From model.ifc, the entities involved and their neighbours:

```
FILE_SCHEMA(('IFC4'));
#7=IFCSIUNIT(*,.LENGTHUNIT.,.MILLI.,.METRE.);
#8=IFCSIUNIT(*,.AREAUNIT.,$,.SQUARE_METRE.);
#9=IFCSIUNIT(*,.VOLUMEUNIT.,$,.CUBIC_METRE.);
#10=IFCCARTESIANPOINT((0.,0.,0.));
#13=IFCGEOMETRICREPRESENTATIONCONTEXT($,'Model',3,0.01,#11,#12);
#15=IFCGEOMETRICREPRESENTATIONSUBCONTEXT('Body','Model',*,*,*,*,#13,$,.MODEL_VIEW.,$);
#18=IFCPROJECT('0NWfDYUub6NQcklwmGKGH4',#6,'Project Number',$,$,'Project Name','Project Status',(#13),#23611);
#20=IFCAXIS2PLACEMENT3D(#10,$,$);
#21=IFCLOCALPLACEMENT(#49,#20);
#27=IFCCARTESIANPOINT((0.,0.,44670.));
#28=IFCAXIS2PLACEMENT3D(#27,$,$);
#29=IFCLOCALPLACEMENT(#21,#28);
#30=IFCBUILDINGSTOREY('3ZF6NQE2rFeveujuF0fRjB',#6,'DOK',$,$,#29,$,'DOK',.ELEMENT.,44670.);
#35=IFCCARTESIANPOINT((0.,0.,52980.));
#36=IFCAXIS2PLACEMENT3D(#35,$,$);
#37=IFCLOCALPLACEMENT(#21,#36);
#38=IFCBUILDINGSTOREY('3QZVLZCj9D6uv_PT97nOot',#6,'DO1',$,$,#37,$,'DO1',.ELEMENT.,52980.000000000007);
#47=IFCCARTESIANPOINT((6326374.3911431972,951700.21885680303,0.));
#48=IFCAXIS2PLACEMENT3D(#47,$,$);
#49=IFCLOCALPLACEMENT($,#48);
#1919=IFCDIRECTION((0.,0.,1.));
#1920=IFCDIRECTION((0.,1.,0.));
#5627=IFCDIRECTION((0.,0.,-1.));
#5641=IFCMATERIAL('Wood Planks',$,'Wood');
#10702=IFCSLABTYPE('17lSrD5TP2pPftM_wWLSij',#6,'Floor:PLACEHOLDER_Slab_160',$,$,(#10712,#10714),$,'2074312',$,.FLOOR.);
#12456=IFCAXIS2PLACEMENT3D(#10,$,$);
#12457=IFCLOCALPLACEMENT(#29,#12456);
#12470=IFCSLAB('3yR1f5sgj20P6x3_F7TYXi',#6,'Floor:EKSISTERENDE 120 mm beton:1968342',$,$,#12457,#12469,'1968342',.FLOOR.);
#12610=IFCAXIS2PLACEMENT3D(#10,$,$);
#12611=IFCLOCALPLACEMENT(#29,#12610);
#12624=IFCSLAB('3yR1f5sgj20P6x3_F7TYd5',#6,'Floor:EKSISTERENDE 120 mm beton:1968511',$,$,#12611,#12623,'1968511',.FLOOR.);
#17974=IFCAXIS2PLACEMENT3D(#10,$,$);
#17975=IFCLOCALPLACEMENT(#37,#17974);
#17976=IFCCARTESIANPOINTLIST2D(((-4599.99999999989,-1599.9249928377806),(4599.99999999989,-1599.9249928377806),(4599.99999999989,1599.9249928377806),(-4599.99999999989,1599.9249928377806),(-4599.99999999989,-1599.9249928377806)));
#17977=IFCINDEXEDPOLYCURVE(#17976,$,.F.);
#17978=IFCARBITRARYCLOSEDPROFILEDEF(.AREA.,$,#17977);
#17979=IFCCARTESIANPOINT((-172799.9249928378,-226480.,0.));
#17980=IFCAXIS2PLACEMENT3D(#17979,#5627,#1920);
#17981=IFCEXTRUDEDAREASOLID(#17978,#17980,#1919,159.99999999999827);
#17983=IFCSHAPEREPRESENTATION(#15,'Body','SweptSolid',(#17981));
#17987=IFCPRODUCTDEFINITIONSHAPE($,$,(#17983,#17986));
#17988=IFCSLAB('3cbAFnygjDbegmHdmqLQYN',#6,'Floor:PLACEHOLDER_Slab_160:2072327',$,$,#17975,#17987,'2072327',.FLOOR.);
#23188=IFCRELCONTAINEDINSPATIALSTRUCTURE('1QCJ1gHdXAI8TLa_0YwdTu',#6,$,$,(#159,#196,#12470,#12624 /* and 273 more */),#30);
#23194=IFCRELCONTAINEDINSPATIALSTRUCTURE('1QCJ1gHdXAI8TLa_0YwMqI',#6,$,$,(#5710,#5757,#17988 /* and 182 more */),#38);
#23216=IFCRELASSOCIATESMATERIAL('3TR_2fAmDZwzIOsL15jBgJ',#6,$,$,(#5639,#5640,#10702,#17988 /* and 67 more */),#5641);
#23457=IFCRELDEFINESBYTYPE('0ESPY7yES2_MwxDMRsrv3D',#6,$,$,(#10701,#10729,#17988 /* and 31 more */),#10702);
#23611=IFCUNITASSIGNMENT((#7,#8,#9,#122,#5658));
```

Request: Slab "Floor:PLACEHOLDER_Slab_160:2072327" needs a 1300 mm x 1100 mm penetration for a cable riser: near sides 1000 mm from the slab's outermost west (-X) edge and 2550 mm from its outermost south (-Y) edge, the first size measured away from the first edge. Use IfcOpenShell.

```python
import numpy as np
import ifcopenshell
import ifcopenshell.api.feature
import ifcopenshell.api.geometry
import ifcopenshell.api.root
import ifcopenshell.geom
import ifcopenshell.util.placement
import ifcopenshell.util.representation
import ifcopenshell.util.shape
import ifcopenshell.util.unit

model = ifcopenshell.open("model.ifc")
unit_scale = ifcopenshell.util.unit.calculate_unit_scale(model)
settings = ifcopenshell.geom.settings()


def volume(element):
    """Net volume in cubic metres, openings subtracted."""
    shape = ifcopenshell.geom.create_shape(settings, element)
    return ifcopenshell.util.shape.get_volume(shape.geometry)


slab = model.by_id(17988)
before = volume(slab)

# Extent in the slab's own axes, in metres. The edges named are its -X and -Y sides.
slab_shape = ifcopenshell.geom.create_shape(settings, slab)
vertices = ifcopenshell.util.shape.get_vertices(slab_shape.geometry)
x_min, y_min, bottom = vertices.min(axis=0)
top = vertices[:, 2].max()

opening = ifcopenshell.api.root.create_entity(model, ifc_class="IfcOpeningElement", name="Cable riser opening", predefined_type="OPENING")
context = ifcopenshell.util.representation.get_context(model, "Model", "Body", "MODEL_VIEW")
width, depth = 1.3, 1.1
outline = [(0.0, 0.0), (width, 0.0), (width, depth), (0.0, depth), (0.0, 0.0)]
# Overshoot both faces by 50 mm so the cut is clean.
shape = ifcopenshell.api.geometry.add_slab_representation(
    model, context=context, depth=top - bottom + 0.1, polyline=outline
)
ifcopenshell.api.geometry.assign_representation(model, product=opening, representation=shape)

matrix = ifcopenshell.util.placement.get_local_placement(slab.ObjectPlacement)
matrix[:, 3] = matrix @ np.append(np.array([x_min + 1, y_min + 2.55, bottom - 0.05]) / unit_scale, 1.0)
ifcopenshell.api.geometry.edit_object_placement(model, product=opening, matrix=matrix, is_si=False)
ifcopenshell.api.feature.add_feature(model, feature=opening, element=slab)

after = volume(slab)

print(f"slab volume {before:.3f} -> {after:.3f} m3")

model.write("model_rev.ifc")
```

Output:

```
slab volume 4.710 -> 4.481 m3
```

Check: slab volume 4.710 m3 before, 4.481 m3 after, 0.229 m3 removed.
